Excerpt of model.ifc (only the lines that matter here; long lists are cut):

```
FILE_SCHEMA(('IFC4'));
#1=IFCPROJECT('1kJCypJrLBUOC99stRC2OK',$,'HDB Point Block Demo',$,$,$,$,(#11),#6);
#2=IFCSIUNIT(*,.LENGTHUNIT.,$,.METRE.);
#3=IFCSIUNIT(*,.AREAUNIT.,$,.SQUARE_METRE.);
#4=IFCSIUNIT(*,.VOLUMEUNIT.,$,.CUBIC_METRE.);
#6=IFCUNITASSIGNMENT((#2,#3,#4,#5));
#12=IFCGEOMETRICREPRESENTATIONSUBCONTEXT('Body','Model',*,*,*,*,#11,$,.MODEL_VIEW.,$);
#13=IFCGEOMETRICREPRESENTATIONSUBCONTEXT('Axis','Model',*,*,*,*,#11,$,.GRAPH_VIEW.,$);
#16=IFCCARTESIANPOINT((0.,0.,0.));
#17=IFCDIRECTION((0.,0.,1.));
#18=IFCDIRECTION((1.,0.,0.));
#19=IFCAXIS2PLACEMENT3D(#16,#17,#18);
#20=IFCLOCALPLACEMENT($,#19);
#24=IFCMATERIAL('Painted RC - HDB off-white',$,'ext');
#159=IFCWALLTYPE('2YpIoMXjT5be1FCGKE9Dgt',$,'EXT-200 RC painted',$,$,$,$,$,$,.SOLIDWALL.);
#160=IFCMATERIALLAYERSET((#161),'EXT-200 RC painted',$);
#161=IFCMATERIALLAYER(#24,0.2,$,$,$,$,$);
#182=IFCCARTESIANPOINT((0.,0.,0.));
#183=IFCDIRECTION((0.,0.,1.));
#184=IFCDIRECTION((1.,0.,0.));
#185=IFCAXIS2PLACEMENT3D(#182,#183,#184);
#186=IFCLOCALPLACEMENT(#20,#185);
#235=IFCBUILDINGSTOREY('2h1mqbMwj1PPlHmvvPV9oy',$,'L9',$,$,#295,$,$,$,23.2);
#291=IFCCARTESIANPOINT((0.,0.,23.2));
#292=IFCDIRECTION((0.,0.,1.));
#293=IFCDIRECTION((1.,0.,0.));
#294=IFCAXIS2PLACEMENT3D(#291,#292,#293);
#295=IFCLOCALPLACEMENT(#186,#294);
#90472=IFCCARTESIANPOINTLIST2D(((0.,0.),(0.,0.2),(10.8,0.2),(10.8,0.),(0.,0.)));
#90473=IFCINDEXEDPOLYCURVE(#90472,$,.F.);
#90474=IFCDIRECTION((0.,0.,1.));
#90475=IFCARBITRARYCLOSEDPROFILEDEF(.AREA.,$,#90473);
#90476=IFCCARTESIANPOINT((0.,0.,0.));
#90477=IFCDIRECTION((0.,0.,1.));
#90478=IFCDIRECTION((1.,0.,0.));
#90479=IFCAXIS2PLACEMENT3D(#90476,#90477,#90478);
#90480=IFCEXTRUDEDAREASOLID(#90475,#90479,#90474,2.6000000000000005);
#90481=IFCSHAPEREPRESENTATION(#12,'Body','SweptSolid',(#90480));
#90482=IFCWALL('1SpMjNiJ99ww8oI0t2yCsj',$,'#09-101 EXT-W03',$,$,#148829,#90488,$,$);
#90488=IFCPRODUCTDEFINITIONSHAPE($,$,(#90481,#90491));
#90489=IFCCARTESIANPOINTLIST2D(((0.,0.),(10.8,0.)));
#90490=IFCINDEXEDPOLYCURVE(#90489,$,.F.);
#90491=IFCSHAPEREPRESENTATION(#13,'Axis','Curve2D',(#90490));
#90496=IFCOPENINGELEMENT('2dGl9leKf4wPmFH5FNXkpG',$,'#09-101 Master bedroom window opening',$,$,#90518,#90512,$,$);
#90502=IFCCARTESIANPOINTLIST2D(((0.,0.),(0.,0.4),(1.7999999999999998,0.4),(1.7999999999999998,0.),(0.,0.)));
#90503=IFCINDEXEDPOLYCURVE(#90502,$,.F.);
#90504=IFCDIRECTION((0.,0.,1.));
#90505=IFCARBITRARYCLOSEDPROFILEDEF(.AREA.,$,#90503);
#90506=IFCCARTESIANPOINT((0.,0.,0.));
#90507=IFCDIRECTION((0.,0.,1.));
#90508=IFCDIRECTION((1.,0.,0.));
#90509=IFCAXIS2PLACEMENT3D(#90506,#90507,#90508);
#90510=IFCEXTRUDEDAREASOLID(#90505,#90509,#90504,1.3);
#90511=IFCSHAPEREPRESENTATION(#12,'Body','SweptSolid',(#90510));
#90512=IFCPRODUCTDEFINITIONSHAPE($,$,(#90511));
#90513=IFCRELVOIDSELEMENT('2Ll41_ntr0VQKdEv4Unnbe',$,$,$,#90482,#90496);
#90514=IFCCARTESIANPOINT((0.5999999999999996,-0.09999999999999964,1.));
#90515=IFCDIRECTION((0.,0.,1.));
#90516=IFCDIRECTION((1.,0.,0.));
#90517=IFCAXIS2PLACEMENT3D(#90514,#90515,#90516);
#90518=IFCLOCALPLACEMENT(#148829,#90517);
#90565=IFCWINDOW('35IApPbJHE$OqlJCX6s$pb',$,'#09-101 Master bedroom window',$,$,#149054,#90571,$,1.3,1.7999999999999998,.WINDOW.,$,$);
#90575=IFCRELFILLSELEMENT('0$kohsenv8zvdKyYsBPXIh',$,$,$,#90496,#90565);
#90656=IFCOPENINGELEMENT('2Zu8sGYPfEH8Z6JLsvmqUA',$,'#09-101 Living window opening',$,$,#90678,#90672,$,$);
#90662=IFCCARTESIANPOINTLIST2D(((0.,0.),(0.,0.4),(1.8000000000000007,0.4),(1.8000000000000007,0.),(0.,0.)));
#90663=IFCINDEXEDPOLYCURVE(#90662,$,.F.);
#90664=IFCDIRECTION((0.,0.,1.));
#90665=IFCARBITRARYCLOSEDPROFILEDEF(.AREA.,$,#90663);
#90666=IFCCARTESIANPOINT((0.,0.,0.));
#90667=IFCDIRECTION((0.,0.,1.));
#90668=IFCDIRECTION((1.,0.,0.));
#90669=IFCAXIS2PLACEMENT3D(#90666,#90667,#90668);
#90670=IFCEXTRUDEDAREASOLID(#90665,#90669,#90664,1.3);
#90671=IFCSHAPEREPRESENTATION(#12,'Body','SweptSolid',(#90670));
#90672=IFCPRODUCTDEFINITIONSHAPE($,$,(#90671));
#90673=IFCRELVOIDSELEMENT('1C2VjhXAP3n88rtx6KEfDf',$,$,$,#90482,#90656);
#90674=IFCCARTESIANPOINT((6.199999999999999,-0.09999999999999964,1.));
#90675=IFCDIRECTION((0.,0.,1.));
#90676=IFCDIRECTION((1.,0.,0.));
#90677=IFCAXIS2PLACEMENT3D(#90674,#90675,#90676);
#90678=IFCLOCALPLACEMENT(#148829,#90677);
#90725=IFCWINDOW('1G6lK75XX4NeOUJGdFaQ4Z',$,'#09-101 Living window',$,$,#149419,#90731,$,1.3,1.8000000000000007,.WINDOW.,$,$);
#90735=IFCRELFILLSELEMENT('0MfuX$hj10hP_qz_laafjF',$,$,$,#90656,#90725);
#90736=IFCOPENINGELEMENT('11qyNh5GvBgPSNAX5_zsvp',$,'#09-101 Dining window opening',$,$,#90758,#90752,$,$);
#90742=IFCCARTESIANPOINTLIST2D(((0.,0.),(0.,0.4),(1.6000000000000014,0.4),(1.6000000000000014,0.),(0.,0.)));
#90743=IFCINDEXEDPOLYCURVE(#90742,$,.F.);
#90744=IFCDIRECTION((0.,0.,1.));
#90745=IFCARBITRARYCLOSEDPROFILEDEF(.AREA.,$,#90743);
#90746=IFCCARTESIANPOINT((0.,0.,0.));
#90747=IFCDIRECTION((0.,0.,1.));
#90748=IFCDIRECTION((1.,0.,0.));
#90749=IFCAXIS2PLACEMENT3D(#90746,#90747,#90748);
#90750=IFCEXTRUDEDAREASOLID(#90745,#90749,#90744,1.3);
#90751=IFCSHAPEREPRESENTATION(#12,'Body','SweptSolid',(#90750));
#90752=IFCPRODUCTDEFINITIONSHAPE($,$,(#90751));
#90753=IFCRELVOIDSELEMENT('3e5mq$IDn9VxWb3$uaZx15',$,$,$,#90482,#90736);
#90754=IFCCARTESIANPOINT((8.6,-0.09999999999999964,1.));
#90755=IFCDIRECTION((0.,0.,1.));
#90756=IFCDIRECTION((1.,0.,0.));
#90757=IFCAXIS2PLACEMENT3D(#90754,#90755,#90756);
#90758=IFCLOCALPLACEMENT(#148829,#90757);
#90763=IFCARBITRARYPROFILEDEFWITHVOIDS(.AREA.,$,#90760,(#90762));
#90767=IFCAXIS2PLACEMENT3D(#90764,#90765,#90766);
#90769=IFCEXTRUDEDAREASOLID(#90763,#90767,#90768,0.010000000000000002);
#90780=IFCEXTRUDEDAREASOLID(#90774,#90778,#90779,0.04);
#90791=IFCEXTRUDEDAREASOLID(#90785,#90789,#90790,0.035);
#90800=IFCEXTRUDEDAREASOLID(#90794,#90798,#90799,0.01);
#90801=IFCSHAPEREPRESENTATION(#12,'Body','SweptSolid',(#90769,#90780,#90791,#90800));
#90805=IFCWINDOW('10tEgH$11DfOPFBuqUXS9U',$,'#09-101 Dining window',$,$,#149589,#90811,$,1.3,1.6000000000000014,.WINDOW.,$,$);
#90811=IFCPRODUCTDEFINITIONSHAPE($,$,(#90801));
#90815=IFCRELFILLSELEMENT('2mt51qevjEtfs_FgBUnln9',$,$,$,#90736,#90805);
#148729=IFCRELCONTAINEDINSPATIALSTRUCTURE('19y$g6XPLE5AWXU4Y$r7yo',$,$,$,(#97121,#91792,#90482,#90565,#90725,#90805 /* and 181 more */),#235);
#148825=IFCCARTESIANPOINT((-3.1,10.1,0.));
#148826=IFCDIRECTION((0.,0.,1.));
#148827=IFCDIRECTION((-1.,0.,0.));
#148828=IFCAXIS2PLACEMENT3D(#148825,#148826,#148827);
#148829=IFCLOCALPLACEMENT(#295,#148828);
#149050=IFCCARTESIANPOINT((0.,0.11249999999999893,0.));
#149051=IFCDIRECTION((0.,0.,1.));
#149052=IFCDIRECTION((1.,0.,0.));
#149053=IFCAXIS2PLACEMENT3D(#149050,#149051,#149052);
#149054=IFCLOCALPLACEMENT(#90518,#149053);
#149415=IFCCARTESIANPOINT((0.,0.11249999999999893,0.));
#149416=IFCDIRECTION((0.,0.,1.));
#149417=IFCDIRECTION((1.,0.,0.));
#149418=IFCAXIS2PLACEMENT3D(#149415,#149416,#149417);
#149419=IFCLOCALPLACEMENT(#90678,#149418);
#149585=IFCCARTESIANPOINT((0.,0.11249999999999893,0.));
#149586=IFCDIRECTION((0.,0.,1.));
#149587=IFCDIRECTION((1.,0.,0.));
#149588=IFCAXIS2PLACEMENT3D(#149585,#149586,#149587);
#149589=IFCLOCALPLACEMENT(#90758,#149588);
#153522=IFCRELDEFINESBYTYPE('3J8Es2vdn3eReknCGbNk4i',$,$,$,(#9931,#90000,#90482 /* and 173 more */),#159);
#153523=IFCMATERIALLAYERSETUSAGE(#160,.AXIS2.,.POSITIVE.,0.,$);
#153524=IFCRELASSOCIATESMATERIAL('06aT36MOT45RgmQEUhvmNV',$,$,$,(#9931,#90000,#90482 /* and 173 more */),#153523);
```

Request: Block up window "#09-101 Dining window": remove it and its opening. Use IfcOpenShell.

```python
import ifcopenshell
import ifcopenshell.api.feature
import ifcopenshell.api.root
import ifcopenshell.geom
import ifcopenshell.util.shape

model = ifcopenshell.open("model.ifc")
settings = ifcopenshell.geom.settings()


def volume(element):
    """Net volume in cubic metres, openings subtracted."""
    shape = ifcopenshell.geom.create_shape(settings, element)
    return ifcopenshell.util.shape.get_volume(shape.geometry)


window = model.by_guid("10tEgH$11DfOPFBuqUXS9U")
opening = window.FillsVoids[0].RelatingOpeningElement
wall = opening.VoidsElements[0].RelatingBuildingElement
before = volume(wall)

ifcopenshell.api.root.remove_product(model, product=window)
ifcopenshell.api.feature.remove_feature(model, feature=opening)

after = volume(wall)

print(f"wall volume {before:.3f} -> {after:.3f} m3")

model.write("model_updated.ifc")
```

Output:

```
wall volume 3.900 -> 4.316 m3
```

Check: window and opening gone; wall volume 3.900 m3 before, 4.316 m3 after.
